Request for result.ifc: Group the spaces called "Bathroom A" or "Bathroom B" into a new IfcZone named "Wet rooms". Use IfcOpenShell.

First a look at what the model holds.

```python
import ifcopenshell

model = ifcopenshell.open("result.ifc")
print(model.schema)
seen = {}
for space in model.by_type("IfcSpace"):
    seen[space.Name] = seen.get(space.Name, 0) + 1
for name, count in sorted(seen.items(), key=str):
    print(count, "x", name)
print("zones:", [z.Name for z in model.by_type("IfcZone")][:20])
```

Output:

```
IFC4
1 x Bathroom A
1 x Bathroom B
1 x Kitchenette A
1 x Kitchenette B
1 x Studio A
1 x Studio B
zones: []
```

```python
import ifcopenshell
import ifcopenshell.api.group
import ifcopenshell.api.root

model = ifcopenshell.open("result.ifc")

names = {"Bathroom A", "Bathroom B"}
spaces = [s for s in model.by_type("IfcSpace") if s.Name in names]

zone = ifcopenshell.api.root.create_entity(model, ifc_class="IfcZone", name="Wet rooms")
ifcopenshell.api.group.assign_group(model, products=spaces, group=zone)
print(len(spaces), "spaces in", zone.Name)

model.write("result_edited.ifc")
```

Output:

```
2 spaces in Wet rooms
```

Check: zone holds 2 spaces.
